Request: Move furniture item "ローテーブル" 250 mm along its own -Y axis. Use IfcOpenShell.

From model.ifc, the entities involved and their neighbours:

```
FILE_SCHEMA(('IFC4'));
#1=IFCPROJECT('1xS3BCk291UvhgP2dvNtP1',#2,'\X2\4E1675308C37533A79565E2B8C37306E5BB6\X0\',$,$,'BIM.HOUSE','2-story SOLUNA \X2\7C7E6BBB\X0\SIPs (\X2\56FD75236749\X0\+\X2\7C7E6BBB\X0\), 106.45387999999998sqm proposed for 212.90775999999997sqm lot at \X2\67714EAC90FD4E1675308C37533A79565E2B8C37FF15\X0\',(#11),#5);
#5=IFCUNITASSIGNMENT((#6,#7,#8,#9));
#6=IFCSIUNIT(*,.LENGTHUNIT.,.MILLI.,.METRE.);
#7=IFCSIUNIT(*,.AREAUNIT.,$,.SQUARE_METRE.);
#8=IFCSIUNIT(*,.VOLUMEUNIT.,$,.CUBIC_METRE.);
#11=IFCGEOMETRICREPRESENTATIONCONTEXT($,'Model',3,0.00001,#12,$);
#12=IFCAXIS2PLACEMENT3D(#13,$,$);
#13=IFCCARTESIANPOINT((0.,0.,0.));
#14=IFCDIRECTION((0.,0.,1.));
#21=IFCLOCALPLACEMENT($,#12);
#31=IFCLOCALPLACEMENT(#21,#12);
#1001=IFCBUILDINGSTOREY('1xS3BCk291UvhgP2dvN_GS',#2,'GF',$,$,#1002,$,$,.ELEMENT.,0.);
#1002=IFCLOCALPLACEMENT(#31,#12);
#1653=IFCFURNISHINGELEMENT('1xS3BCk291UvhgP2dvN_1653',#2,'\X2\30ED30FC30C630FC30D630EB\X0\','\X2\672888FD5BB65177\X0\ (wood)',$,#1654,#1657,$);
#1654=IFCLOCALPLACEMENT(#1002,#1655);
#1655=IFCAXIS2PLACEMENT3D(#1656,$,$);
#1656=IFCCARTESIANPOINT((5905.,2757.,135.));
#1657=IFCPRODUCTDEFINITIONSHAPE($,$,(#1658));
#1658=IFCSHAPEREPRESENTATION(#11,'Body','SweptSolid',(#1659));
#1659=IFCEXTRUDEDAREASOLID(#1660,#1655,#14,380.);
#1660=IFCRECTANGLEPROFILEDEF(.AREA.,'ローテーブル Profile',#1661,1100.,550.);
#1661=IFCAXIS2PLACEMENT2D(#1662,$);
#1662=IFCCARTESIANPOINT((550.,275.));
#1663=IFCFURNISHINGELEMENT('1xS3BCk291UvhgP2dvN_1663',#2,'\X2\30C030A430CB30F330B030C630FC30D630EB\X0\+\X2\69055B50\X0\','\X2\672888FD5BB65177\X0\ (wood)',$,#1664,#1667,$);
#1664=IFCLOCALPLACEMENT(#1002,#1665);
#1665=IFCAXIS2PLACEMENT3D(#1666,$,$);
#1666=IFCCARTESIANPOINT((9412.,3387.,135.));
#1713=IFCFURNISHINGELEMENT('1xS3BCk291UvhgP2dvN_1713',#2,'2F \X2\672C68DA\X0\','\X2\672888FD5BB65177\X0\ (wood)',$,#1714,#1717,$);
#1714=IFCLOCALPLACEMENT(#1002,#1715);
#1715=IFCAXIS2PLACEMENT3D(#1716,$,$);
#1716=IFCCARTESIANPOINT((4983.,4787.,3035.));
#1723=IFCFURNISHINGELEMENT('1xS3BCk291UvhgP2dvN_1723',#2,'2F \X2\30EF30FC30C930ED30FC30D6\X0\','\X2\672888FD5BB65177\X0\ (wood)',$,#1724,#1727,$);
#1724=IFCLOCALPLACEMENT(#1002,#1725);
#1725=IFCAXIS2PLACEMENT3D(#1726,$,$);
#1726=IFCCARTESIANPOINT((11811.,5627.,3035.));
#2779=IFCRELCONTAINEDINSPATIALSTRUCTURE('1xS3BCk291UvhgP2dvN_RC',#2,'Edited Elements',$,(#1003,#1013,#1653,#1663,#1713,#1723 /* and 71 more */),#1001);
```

```python
import ifcopenshell
import ifcopenshell.api.geometry
import ifcopenshell.util.placement
import ifcopenshell.util.unit

model = ifcopenshell.open("model.ifc")
unit_scale = ifcopenshell.util.unit.calculate_unit_scale(model)

item = model.by_guid("1xS3BCk291UvhgP2dvN_1653")
matrix = ifcopenshell.util.placement.get_local_placement(item.ObjectPlacement)
matrix[:3, 3] -= matrix[:3, 1] * 0.25 / unit_scale
ifcopenshell.api.geometry.edit_object_placement(model, product=item, matrix=matrix, is_si=False)

print(ifcopenshell.util.placement.get_local_placement(item.ObjectPlacement).round(3) + 0.0)

model.write("model-out.ifc")
```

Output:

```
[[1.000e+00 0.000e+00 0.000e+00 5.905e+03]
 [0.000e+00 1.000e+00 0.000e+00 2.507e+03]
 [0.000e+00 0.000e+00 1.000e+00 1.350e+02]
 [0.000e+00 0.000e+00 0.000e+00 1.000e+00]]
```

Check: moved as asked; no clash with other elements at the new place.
